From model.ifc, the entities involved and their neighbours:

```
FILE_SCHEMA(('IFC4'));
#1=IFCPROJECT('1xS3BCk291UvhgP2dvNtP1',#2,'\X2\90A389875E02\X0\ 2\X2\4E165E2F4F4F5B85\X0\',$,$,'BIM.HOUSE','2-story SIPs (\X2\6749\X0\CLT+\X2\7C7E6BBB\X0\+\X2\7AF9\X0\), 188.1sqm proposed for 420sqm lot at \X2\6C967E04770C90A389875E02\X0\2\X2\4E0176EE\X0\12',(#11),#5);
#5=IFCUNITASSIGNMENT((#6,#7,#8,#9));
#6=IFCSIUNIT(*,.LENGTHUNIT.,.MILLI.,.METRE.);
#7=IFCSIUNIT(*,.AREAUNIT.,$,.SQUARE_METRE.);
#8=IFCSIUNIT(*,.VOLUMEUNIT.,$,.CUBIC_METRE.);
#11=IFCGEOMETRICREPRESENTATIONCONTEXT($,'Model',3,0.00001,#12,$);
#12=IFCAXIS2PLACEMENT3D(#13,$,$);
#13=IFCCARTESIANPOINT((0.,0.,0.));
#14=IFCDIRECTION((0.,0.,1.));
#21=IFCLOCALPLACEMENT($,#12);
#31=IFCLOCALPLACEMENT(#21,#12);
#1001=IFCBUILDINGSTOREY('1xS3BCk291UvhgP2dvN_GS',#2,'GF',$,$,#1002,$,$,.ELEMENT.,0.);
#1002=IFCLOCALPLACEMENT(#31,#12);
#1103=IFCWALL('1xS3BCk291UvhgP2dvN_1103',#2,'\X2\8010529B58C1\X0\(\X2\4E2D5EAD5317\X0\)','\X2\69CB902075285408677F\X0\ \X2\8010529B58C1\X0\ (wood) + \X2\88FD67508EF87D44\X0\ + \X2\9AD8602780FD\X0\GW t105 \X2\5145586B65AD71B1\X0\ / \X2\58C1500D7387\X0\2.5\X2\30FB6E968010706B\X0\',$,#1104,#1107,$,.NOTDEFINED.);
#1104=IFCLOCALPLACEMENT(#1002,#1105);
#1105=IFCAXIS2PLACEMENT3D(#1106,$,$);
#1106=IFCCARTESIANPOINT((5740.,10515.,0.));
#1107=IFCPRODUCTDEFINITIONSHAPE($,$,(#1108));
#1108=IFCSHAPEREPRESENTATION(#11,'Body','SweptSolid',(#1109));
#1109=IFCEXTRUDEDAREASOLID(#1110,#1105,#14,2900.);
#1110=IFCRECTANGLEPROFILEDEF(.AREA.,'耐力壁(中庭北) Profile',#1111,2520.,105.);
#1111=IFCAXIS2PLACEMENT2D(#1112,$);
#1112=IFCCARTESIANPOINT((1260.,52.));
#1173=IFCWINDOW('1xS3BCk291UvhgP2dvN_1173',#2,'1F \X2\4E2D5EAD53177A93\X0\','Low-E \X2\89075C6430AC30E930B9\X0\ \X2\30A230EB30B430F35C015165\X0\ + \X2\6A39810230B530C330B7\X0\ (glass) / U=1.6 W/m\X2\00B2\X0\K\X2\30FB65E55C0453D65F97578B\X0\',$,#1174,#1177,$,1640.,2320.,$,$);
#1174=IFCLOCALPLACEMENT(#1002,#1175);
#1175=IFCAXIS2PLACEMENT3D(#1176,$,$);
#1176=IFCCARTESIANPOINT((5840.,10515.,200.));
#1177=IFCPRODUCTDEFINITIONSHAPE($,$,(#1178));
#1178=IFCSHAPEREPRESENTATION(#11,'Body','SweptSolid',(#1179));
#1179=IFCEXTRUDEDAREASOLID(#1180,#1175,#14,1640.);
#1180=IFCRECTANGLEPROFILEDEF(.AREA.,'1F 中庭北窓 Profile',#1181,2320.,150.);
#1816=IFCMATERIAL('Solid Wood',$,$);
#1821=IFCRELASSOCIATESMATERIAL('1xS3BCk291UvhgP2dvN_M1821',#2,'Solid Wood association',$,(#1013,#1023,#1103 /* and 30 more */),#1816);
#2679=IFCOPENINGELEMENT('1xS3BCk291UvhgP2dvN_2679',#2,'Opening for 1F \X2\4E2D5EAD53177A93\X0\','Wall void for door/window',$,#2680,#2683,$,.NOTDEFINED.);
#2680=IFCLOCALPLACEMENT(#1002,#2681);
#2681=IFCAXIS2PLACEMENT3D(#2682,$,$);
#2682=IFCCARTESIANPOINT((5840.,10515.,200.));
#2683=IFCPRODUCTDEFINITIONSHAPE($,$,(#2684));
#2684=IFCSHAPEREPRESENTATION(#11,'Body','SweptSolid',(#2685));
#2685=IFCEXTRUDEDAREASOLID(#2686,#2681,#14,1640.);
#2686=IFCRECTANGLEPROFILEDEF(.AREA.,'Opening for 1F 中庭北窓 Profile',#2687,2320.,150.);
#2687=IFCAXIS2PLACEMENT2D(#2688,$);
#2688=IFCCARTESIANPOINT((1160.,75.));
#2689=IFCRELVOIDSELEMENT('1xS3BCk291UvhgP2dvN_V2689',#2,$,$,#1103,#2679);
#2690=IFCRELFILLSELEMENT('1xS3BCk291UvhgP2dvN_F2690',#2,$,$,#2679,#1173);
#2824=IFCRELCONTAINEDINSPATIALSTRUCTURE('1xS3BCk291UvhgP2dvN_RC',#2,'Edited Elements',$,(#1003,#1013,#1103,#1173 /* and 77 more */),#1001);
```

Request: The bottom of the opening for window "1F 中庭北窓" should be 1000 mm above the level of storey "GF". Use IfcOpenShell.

```python
import numpy as np
import ifcopenshell
import ifcopenshell.api.geometry
import ifcopenshell.geom
import ifcopenshell.util.element
import ifcopenshell.util.placement
import ifcopenshell.util.shape
import ifcopenshell.util.unit

model = ifcopenshell.open("model.ifc")
unit_scale = ifcopenshell.util.unit.calculate_unit_scale(model)

window = model.by_id(1173)
opening = window.FillsVoids[0].RelatingOpeningElement
storey = ifcopenshell.util.element.get_container(window, ifc_class="IfcBuildingStorey")
level = ifcopenshell.util.placement.get_local_placement(storey.ObjectPlacement)[2, 3]

# The opening's origin need not be at the sill, so measure its lowest point.
shape = ifcopenshell.geom.create_shape(ifcopenshell.geom.settings(), opening)
bottom = ifcopenshell.util.shape.get_shape_bottom_elevation(shape, shape.geometry) / unit_scale
dz = level + 1 / unit_scale - bottom

shift = np.array([0.0, 0.0, dz])
# The window is not placed relative to its opening, so move both.
for product in (opening, window):
    matrix = ifcopenshell.util.placement.get_local_placement(product.ObjectPlacement)
    matrix[:3, 3] += shift
    ifcopenshell.api.geometry.edit_object_placement(model, product=product, matrix=matrix, is_si=False)

print(f"moved by {dz * unit_scale:+.3f} m")

model.write("model_updated.ifc")
```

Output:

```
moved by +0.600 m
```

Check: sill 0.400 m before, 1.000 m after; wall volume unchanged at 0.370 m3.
